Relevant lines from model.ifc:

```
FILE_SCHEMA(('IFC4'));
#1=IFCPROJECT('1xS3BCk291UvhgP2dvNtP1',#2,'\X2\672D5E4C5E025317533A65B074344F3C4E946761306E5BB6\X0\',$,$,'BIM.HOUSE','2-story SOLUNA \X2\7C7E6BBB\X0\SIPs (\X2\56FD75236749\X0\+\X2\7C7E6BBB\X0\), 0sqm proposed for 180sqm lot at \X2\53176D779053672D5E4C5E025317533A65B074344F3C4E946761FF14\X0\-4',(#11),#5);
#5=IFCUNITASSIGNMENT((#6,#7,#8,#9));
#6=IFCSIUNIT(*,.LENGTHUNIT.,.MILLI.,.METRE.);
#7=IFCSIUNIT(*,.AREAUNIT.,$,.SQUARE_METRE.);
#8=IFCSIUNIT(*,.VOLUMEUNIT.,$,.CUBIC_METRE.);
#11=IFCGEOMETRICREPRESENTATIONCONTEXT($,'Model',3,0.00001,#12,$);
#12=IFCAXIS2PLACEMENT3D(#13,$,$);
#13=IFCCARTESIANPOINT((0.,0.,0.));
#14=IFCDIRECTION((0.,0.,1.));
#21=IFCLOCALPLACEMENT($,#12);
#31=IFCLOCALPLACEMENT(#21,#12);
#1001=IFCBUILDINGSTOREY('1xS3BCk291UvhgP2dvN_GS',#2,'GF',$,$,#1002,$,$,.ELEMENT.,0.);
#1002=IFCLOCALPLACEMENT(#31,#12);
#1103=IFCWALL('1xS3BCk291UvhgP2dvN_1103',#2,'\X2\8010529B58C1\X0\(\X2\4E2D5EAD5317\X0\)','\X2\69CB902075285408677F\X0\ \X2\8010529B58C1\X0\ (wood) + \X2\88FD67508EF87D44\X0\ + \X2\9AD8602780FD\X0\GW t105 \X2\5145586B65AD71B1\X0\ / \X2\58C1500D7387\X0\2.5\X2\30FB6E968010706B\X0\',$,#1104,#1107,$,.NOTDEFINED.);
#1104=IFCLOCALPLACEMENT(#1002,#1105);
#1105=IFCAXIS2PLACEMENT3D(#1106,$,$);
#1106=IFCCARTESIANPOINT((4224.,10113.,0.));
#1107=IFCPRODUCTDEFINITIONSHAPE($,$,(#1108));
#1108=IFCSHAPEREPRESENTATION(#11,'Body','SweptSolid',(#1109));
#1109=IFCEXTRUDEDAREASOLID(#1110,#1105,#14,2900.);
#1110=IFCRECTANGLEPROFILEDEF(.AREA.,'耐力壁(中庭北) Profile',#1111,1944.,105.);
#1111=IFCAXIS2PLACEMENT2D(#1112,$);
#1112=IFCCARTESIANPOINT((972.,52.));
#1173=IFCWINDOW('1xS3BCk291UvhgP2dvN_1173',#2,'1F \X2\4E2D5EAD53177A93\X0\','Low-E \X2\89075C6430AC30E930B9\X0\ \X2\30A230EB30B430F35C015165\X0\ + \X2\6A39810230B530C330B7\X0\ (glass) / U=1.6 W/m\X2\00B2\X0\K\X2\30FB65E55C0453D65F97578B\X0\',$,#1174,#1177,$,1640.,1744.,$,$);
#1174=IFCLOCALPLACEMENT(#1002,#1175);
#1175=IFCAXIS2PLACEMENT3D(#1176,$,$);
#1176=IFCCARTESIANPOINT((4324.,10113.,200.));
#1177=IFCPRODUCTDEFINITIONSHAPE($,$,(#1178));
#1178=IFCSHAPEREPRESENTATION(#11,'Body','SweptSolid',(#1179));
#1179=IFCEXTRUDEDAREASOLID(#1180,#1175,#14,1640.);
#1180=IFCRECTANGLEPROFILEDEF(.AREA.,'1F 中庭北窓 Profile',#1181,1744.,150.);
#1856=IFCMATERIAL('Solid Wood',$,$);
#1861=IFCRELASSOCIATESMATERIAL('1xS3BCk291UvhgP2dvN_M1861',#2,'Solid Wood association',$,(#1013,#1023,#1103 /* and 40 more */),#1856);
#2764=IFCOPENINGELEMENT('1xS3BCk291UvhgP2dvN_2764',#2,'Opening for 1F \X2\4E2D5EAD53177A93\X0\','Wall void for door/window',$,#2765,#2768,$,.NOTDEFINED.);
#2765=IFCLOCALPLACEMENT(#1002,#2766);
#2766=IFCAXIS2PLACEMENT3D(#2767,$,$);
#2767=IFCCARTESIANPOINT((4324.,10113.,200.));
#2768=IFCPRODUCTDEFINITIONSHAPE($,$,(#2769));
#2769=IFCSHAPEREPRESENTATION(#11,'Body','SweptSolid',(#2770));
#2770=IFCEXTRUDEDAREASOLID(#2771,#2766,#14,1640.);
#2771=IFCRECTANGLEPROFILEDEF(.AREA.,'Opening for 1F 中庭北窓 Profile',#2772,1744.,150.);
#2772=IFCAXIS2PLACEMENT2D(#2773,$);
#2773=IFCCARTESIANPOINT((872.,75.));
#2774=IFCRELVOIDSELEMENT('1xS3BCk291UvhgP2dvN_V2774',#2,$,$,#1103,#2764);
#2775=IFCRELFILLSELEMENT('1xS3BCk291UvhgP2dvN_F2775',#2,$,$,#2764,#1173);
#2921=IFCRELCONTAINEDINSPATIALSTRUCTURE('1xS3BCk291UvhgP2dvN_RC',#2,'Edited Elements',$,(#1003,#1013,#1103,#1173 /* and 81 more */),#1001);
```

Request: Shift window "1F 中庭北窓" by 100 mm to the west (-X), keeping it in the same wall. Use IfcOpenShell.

```python
import ifcopenshell
import ifcopenshell.api.geometry
import ifcopenshell.util.placement

model = ifcopenshell.open("model.ifc")

window = model.by_id(1173)
opening = window.FillsVoids[0].RelatingOpeningElement
wall = opening.VoidsElements[0].RelatingBuildingElement

wall_matrix = ifcopenshell.util.placement.get_local_placement(wall.ObjectPlacement)
shift = wall_matrix[:3, 0] * -100.0
before = ifcopenshell.util.placement.get_local_placement(window.ObjectPlacement)[:3, 3].copy()

# The window is not placed relative to its opening, so move both.
for product in (opening, window):
    matrix = ifcopenshell.util.placement.get_local_placement(product.ObjectPlacement)
    matrix[:3, 3] += shift
    ifcopenshell.api.geometry.edit_object_placement(model, product=product, matrix=matrix, is_si=False)

after = ifcopenshell.util.placement.get_local_placement(window.ObjectPlacement)[:3, 3]
print("window moved by", (after - before).round(3) + 0.0)

model.write("model_updated.ifc")
```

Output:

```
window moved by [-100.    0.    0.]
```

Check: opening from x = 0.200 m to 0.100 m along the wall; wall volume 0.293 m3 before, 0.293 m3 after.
